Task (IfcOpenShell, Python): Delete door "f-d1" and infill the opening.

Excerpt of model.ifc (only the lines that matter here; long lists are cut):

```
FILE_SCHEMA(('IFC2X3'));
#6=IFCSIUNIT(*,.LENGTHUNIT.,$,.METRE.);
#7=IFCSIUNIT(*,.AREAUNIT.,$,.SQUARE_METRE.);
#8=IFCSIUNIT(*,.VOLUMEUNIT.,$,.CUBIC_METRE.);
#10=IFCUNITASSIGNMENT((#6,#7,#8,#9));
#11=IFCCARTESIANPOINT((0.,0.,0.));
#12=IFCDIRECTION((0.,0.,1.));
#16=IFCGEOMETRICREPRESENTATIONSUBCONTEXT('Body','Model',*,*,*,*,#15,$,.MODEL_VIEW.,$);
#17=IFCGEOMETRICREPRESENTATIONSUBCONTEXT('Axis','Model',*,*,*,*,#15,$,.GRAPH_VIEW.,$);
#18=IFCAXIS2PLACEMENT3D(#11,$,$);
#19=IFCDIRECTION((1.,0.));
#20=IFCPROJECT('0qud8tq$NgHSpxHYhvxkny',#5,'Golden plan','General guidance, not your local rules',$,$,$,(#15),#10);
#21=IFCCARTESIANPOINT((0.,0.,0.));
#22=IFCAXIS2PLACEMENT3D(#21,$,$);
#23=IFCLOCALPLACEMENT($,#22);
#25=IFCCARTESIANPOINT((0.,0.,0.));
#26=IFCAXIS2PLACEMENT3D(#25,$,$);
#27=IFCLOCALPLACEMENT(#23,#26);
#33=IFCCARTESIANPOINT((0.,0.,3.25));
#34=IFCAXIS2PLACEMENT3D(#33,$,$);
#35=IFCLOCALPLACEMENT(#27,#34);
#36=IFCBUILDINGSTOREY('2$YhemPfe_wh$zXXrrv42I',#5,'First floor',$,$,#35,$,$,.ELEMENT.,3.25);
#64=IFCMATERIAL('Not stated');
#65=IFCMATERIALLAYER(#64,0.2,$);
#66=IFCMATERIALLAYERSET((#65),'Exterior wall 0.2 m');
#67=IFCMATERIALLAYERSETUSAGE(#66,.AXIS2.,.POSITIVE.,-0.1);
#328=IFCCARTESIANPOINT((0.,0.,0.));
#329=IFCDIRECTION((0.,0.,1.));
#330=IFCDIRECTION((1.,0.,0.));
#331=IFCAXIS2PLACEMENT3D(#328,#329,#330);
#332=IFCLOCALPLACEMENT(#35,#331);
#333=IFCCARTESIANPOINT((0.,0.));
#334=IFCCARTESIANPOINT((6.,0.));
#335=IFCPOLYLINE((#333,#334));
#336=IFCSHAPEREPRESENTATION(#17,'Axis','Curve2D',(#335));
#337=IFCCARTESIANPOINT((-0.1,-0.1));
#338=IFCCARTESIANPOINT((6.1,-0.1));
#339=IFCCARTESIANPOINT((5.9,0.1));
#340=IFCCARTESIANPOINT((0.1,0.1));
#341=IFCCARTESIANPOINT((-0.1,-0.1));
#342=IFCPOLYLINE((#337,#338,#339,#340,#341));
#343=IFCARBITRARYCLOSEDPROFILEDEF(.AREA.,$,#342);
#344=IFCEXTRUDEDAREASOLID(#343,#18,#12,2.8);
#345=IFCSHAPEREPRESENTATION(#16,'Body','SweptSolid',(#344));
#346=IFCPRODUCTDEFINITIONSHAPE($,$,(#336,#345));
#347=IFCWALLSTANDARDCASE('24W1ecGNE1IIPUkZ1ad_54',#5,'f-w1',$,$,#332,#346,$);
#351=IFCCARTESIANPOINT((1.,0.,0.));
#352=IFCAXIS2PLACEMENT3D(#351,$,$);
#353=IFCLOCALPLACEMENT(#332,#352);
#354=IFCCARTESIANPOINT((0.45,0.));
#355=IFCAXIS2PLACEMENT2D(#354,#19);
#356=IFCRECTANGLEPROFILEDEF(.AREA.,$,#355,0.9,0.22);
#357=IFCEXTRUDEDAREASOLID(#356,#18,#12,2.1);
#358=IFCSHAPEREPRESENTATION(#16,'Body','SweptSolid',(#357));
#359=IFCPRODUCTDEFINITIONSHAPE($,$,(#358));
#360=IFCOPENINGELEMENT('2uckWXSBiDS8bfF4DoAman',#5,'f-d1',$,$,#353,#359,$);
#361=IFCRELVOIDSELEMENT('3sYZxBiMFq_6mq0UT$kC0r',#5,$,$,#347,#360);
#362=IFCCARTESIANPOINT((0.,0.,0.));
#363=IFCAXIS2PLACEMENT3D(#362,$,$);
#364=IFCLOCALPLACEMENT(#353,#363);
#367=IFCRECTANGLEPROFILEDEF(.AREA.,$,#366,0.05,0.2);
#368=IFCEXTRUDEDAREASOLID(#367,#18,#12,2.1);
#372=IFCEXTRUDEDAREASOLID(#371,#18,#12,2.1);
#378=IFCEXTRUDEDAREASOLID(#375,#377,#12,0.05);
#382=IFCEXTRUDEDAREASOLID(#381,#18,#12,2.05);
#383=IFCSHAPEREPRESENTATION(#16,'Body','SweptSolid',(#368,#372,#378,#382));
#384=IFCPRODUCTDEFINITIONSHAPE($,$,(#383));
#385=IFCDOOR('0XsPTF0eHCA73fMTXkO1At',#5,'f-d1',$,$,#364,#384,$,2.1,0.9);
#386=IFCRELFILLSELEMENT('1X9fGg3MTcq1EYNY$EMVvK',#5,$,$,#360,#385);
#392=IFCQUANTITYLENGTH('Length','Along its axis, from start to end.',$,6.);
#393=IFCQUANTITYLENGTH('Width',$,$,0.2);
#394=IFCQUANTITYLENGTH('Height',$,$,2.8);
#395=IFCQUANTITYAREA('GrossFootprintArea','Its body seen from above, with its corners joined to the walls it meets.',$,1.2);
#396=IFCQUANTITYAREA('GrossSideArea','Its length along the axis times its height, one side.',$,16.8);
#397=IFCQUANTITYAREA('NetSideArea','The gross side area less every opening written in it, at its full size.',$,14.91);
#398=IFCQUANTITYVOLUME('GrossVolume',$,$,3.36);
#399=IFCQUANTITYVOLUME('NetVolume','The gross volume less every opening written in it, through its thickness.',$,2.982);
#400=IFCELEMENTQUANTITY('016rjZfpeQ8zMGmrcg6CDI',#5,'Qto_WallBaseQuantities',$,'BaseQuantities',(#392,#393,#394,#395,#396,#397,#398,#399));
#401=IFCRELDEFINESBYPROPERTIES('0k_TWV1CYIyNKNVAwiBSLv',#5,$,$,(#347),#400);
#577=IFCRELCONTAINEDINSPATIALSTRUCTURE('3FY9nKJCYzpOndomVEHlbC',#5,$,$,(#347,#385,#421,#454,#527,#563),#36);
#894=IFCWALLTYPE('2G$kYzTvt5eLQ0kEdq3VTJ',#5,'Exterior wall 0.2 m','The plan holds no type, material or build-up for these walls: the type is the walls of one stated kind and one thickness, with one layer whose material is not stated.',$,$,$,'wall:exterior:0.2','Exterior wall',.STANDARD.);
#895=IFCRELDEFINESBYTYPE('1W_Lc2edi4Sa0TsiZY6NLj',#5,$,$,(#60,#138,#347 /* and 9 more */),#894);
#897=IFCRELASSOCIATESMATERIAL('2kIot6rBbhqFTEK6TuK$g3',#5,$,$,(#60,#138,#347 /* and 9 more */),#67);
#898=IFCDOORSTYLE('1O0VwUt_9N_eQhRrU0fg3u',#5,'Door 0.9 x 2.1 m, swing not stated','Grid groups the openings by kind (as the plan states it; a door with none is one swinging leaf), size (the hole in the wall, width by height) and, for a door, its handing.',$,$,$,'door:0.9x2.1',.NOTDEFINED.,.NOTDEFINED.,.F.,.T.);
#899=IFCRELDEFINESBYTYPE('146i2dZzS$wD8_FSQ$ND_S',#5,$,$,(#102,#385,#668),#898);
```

```python
import ifcopenshell
import ifcopenshell.api.feature
import ifcopenshell.api.pset
import ifcopenshell.api.root
import ifcopenshell.geom
import ifcopenshell.util.element
import ifcopenshell.util.shape
import ifcopenshell.util.unit

model = ifcopenshell.open("model.ifc")
area_scale = ifcopenshell.util.unit.calculate_unit_scale(model, "AREAUNIT")
volume_scale = ifcopenshell.util.unit.calculate_unit_scale(model, "VOLUMEUNIT")
settings = ifcopenshell.geom.settings()


def volume(element):
    """Net volume in cubic metres, openings subtracted."""
    shape = ifcopenshell.geom.create_shape(settings, element)
    return ifcopenshell.util.shape.get_volume(shape.geometry)


door = model.by_guid("0XsPTF0eHCA73fMTXkO1At")
opening = door.FillsVoids[0].RelatingOpeningElement
wall = opening.VoidsElements[0].RelatingBuildingElement
before = volume(wall)

ifcopenshell.api.root.remove_product(model, product=door)
ifcopenshell.api.feature.remove_feature(model, feature=opening)

after = volume(wall)
thickness = 0.2  # wall thickness in metres

# Update the wall's stored quantities.
qto = model.by_id(ifcopenshell.util.element.get_pset(wall, "Qto_WallBaseQuantities", should_inherit=False)["id"])
ifcopenshell.api.pset.edit_qto(model, qto=qto, properties={
    "NetSideArea": after / thickness / area_scale,
    "NetVolume": after / volume_scale,
})

print(f"wall volume {before:.3f} -> {after:.3f} m3")

model.write("model_edited.ifc")
```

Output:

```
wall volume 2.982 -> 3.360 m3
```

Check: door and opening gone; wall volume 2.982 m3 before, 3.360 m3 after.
